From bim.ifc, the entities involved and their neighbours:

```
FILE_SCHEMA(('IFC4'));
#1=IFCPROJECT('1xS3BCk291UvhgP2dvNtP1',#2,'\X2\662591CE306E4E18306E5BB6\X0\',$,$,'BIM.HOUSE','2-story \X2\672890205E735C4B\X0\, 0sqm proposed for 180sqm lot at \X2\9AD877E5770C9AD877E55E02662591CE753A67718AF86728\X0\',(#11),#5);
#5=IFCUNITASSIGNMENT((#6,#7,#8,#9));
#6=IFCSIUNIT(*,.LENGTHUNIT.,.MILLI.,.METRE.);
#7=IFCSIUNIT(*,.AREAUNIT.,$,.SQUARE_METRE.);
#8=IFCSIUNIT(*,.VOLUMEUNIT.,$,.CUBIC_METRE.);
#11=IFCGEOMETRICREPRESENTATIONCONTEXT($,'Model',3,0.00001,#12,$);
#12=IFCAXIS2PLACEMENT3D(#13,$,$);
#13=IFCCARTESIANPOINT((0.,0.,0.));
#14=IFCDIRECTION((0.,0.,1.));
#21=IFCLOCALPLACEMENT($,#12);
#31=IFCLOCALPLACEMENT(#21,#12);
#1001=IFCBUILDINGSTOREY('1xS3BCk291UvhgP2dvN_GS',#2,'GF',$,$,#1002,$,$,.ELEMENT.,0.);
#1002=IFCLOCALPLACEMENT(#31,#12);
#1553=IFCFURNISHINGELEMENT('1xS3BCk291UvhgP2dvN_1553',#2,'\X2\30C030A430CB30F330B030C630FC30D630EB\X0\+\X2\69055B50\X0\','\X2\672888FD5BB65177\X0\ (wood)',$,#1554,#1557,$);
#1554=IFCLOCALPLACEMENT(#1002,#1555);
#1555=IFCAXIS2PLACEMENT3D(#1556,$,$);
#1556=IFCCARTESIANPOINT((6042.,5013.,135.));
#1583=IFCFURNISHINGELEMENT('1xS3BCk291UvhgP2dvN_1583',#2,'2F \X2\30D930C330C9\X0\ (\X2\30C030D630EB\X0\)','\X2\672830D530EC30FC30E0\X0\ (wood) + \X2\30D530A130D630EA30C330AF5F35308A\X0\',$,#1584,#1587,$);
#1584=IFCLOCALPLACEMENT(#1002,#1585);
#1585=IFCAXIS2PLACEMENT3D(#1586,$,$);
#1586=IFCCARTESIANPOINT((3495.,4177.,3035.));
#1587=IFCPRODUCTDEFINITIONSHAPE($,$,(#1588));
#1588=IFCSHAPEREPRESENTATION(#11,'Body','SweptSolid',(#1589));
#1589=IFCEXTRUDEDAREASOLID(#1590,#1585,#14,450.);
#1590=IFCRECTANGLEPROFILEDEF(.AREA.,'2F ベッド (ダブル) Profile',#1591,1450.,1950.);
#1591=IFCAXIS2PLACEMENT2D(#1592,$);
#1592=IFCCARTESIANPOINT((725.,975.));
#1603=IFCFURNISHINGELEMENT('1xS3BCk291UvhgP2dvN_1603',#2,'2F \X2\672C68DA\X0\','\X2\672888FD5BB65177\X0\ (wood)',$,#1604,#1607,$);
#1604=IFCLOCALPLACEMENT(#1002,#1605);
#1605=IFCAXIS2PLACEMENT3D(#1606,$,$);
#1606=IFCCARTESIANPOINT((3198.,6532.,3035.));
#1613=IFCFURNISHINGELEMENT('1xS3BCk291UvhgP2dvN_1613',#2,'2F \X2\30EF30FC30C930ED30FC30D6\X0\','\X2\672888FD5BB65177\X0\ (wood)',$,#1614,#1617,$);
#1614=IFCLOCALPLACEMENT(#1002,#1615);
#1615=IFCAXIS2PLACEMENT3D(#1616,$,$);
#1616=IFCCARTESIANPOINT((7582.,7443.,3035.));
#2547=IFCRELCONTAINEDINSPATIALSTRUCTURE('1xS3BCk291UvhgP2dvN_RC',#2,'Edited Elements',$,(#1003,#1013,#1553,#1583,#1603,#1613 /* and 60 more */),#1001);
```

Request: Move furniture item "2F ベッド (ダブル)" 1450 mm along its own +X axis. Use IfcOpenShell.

```python
import ifcopenshell
import ifcopenshell.api.geometry
import ifcopenshell.util.placement
import ifcopenshell.util.unit

model = ifcopenshell.open("bim.ifc")
unit_scale = ifcopenshell.util.unit.calculate_unit_scale(model)

item = model.by_guid("1xS3BCk291UvhgP2dvN_1583")
matrix = ifcopenshell.util.placement.get_local_placement(item.ObjectPlacement)
matrix[:3, 3] += matrix[:3, 0] * 1.45 / unit_scale
ifcopenshell.api.geometry.edit_object_placement(model, product=item, matrix=matrix, is_si=False)

print(ifcopenshell.util.placement.get_local_placement(item.ObjectPlacement).round(3) + 0.0)

model.write("bim_edited.ifc")
```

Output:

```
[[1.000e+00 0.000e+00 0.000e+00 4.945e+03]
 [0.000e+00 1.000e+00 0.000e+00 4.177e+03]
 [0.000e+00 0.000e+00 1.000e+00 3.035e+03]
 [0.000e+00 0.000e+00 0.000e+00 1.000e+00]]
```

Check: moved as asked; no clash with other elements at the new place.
